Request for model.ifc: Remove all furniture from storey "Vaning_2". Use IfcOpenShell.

First a look at what the model holds.

```python
import ifcopenshell
import ifcopenshell.util.element

model = ifcopenshell.open("model.ifc")
print(model.schema)
storey = next(s for s in model.by_type("IfcBuildingStorey") if s.Name == "Vaning_2")
furniture = [e for e in ifcopenshell.util.element.get_decomposition(storey) if e.is_a("IfcFurnishingElement")]
seen = {}
for e in furniture:
    element_type = ifcopenshell.util.element.get_type(e)
    name = element_type.Name if element_type not in (None, e) else None
    seen[name] = seen.get(name, 0) + 1
for name, count in sorted(seen.items(), key=str):
    print(count, "x", name)
```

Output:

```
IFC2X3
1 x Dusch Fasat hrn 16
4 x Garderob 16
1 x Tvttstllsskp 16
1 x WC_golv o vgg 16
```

```python
import ifcopenshell
import ifcopenshell.api.root
import ifcopenshell.util.element

model = ifcopenshell.open("model.ifc")

storey = next(s for s in model.by_type("IfcBuildingStorey") if s.Name == "Vaning_2")
furniture = [e for e in ifcopenshell.util.element.get_decomposition(storey) if e.is_a("IfcFurnishingElement")]

for e in furniture:
    ifcopenshell.api.root.remove_product(model, product=e)
print(len(furniture), "removed")

model.write("model_rev.ifc")
```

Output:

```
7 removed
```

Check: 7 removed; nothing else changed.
